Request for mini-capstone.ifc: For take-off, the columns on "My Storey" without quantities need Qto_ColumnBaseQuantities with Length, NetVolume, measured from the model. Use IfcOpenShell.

First a look at what the model holds.

```python
import ifcopenshell
import ifcopenshell.util.element
import ifcopenshell.util.unit

model = ifcopenshell.open("mini-capstone.ifc")
print(model.schema)
for unit_type in ("LENGTHUNIT", "AREAUNIT", "VOLUMEUNIT"):
    print(unit_type, ifcopenshell.util.unit.calculate_unit_scale(model, unit_type))
storey = next(s for s in model.by_type("IfcBuildingStorey") if s.Name == "My Storey")
columns = [e for e in ifcopenshell.util.element.get_decomposition(storey) if e.is_a("IfcColumn")]
for e in sorted(columns, key=lambda e: e.id()):
    print(e.id(), e.is_a(), e.Name, list(ifcopenshell.util.element.get_psets(e, qtos_only=True)), sep=" | ")
```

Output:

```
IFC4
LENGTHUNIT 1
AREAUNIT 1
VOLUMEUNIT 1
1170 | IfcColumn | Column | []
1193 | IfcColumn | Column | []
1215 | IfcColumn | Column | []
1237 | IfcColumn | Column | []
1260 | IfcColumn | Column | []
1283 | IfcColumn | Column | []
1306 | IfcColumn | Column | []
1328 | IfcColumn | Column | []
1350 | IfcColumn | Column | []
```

```python
import ifcopenshell
import ifcopenshell.api.pset
import ifcopenshell.geom
import ifcopenshell.util.element
import ifcopenshell.util.shape
import ifcopenshell.util.unit

model = ifcopenshell.open("mini-capstone.ifc")
unit_scale = ifcopenshell.util.unit.calculate_unit_scale(model)
volume_scale = ifcopenshell.util.unit.calculate_unit_scale(model, "VOLUMEUNIT")
settings = ifcopenshell.geom.settings()

storey = next(s for s in model.by_type("IfcBuildingStorey") if s.Name == "My Storey")
columns = [e for e in ifcopenshell.util.element.get_decomposition(storey) if e.is_a("IfcColumn")]

for e in sorted(columns, key=lambda e: e.id()):
    if ifcopenshell.util.element.get_psets(e, qtos_only=True, should_inherit=False):
        continue
    # Geometry comes back in metres, in the element's own axes.
    shape = ifcopenshell.geom.create_shape(settings, e)
    values = {
        "Length": ifcopenshell.util.shape.get_z(shape.geometry) / unit_scale,
        "NetVolume": ifcopenshell.util.shape.get_volume(shape.geometry) / volume_scale,
    }
    qto = ifcopenshell.api.pset.add_qto(model, product=e, name="Qto_ColumnBaseQuantities")
    ifcopenshell.api.pset.edit_qto(model, qto=qto, properties=values)
    print(e.id(), {k: round(v, 3) for k, v in values.items()})

model.write("mini-capstone_updated.ifc")
```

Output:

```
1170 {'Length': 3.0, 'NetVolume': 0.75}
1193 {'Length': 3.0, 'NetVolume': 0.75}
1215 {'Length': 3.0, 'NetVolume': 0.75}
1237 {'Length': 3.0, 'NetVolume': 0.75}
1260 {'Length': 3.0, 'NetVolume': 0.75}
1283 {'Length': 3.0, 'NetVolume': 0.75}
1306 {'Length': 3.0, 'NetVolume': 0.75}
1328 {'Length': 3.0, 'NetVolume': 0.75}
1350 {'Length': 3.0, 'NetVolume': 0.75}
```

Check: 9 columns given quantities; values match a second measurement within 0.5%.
